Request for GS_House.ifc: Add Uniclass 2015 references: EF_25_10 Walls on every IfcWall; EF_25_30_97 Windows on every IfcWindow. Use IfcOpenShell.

First a look at what the model holds.

```python
import ifcopenshell

model = ifcopenshell.open("GS_House.ifc")
print(model.schema)
print("classifications:", [c.Name for c in model.by_type("IfcClassification")])
for ifc_class in ("IfcDoor", "IfcRoof", "IfcStair", "IfcWall", "IfcWindow"):
    print(ifc_class, len(model.by_type(ifc_class)))
```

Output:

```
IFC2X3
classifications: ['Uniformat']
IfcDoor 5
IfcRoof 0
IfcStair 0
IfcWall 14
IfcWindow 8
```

```python
import ifcopenshell
import ifcopenshell.api.classification

model = ifcopenshell.open("GS_House.ifc")

# IFC2X3 requires Source and Edition and has no link from the project to the system.
system = model.create_entity("IfcClassification", Source="NBS", Edition="2015", Name="Uniclass 2015")

codes = {
    "IfcWall": ("EF_25_10", "Walls"),
    "IfcWindow": ("EF_25_30_97", "Windows"),
}
for ifc_class, (code, name) in codes.items():
    products = model.by_type(ifc_class)
    ifcopenshell.api.classification.add_reference(
        model, products=products, classification=system, identification=code, name=name
    )
    print(code, len(products))

model.write("GS_House_v2.ifc")
```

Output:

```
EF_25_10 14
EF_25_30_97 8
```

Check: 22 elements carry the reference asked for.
